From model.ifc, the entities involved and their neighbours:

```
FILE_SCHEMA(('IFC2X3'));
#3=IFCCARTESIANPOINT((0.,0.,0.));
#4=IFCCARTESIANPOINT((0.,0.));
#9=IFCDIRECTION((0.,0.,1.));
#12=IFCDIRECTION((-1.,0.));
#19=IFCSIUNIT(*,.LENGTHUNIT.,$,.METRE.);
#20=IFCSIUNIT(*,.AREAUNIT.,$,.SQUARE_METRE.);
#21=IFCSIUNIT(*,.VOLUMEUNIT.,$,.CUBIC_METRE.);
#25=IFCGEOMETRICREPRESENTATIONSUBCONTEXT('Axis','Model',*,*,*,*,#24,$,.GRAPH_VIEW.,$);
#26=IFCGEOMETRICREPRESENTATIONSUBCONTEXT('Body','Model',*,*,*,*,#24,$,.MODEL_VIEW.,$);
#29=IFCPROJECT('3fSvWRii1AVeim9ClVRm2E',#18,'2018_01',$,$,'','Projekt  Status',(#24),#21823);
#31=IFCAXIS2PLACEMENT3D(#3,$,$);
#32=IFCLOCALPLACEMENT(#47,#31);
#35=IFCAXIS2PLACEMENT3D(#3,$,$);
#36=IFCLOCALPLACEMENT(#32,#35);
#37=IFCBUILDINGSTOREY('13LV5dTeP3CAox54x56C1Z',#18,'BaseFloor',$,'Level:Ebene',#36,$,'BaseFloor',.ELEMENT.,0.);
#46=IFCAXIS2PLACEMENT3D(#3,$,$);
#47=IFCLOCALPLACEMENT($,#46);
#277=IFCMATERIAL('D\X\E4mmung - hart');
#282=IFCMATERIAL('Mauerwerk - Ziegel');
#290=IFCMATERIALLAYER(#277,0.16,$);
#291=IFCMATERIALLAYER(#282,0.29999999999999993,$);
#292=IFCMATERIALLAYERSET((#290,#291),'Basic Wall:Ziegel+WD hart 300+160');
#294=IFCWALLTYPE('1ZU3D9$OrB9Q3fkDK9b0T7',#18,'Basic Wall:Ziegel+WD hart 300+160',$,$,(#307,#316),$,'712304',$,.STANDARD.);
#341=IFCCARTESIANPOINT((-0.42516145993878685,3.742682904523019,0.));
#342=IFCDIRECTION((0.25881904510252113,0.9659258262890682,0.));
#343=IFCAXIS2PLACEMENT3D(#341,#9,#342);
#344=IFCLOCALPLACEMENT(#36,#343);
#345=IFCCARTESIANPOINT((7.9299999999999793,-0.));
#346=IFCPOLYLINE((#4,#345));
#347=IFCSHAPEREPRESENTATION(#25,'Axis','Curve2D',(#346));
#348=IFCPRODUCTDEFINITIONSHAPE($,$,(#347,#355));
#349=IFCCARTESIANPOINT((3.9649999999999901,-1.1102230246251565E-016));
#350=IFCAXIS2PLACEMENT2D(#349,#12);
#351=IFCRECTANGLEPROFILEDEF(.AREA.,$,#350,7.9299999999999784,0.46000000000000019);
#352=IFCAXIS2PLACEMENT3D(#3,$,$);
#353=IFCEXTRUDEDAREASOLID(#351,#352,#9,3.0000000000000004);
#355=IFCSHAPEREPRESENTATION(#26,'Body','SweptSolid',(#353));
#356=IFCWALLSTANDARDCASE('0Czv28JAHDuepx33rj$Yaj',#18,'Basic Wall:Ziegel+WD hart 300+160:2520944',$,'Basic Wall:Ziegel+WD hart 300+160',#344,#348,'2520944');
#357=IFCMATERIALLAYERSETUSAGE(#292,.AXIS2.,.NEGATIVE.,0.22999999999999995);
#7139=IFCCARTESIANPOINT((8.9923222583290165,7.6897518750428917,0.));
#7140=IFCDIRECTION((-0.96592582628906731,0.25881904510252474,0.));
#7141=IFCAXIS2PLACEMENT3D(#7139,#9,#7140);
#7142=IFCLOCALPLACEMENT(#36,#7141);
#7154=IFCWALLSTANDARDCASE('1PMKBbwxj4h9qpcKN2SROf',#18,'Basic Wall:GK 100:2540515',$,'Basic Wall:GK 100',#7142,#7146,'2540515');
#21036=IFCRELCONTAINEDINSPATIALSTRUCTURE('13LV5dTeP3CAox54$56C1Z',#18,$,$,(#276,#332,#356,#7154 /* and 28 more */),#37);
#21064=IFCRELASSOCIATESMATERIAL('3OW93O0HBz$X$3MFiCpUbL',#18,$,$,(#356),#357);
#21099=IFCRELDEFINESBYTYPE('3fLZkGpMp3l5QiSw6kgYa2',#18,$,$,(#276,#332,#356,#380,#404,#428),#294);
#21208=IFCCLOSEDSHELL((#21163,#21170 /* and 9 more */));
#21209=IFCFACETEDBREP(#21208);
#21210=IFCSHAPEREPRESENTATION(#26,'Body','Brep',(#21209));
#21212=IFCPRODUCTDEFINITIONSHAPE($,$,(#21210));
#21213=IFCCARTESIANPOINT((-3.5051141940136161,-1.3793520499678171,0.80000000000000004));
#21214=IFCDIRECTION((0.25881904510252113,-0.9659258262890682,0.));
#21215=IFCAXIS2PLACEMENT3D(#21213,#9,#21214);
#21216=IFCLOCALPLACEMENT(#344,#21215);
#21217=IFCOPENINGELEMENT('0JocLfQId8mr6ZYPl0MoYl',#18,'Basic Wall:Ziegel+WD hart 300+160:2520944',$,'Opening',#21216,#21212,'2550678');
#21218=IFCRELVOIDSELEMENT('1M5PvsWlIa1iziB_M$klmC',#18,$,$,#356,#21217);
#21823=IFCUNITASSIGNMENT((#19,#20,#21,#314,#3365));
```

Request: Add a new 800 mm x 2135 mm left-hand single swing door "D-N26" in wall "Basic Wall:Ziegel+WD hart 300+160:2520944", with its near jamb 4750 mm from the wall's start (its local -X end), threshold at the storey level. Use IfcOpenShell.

```python
import numpy as np
import ifcopenshell
import ifcopenshell.api.feature
import ifcopenshell.api.geometry
import ifcopenshell.api.root
import ifcopenshell.api.spatial
import ifcopenshell.api.type
import ifcopenshell.geom
import ifcopenshell.util.element
import ifcopenshell.util.placement
import ifcopenshell.util.representation
import ifcopenshell.util.shape
import ifcopenshell.util.unit

model = ifcopenshell.open("model.ifc")
unit_scale = ifcopenshell.util.unit.calculate_unit_scale(model)
settings = ifcopenshell.geom.settings()


def volume(element):
    """Net volume in cubic metres, openings subtracted."""
    shape = ifcopenshell.geom.create_shape(settings, element)
    return ifcopenshell.util.shape.get_volume(shape.geometry)


wall = model.by_guid("0Czv28JAHDuepx33rj$Yaj")
storey = ifcopenshell.util.element.get_container(wall, ifc_class="IfcBuildingStorey")
context = ifcopenshell.util.representation.get_context(model, "Model", "Body", "MODEL_VIEW")
before = volume(wall)

width, height, from_end, sill = 0.8, 2.135, 4.75, 0.0  # metres

# The wall runs along its own X axis, and the end named is its -X end.
wall_shape = ifcopenshell.geom.create_shape(settings, wall)
x, y, z = ifcopenshell.util.shape.get_vertices(wall_shape.geometry).T
start = x.min() + from_end
face, thickness = float(y.min()), float(y.max() - y.min())
wall_matrix = ifcopenshell.util.placement.get_local_placement(wall.ObjectPlacement)
level = ifcopenshell.util.placement.get_local_placement(storey.ObjectPlacement)[2, 3]


def in_wall(x, y):
    """Placement at x, y metres in the wall's axes, at sill height."""
    matrix = wall_matrix.copy()
    matrix[:, 3] = wall_matrix @ np.array([x / unit_scale, y / unit_scale, 0.0, 1.0])
    matrix[2, 3] = level + sill / unit_scale
    return matrix


# Opening: a box that overshoots both wall faces by 50 mm.
opening = ifcopenshell.api.root.create_entity(model, ifc_class="IfcOpeningElement")
box = ifcopenshell.api.geometry.add_wall_representation(
    model, context=context, length=width, height=height, thickness=thickness + 0.1
)
ifcopenshell.api.geometry.assign_representation(model, product=opening, representation=box)
ifcopenshell.api.geometry.edit_object_placement(model, product=opening, matrix=in_wall(start, face - 0.05), is_si=False)
ifcopenshell.api.feature.add_feature(model, feature=opening, element=wall)

door = ifcopenshell.api.root.create_entity(model, ifc_class="IfcDoor", name="D-N26")
door.OverallWidth, door.OverallHeight = width / unit_scale, height / unit_scale
body = ifcopenshell.api.geometry.add_door_representation(
    model,
    context=context,
    overall_width=door.OverallWidth,
    overall_height=door.OverallHeight,
    operation_type="SINGLE_SWING_LEFT",
    lining_properties={"LiningDepth": thickness / unit_scale, "ThresholdDepth": thickness / unit_scale},
)
ifcopenshell.api.geometry.assign_representation(model, product=door, representation=body)
ifcopenshell.api.spatial.assign_container(model, products=[door], relating_structure=storey)
fills = ifcopenshell.api.feature.add_filling(model, opening=opening, element=door)
fills.OwnerHistory = door.OwnerHistory  # required in IFC2X3

# IFC2X3 keeps the operation on the door style.
style = ifcopenshell.api.root.create_entity(model, ifc_class="IfcDoorStyle", name="D-N26")
style.OperationType, style.ConstructionType = "SINGLE_SWING_LEFT", "NOTDEFINED"
style.ParameterTakesPrecedence = style.Sizeable = False
ifcopenshell.api.type.assign_type(model, related_objects=[door], relating_type=style)

# The lining spans the wall, so the door starts at the wall face.
ifcopenshell.api.geometry.edit_object_placement(model, product=door, matrix=in_wall(start, face), is_si=False)

after = volume(wall)

print(f"wall volume {before:.3f} -> {after:.3f} m3")

model.write("model_rev.ifc")
```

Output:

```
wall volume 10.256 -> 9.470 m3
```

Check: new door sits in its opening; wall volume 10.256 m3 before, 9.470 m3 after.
